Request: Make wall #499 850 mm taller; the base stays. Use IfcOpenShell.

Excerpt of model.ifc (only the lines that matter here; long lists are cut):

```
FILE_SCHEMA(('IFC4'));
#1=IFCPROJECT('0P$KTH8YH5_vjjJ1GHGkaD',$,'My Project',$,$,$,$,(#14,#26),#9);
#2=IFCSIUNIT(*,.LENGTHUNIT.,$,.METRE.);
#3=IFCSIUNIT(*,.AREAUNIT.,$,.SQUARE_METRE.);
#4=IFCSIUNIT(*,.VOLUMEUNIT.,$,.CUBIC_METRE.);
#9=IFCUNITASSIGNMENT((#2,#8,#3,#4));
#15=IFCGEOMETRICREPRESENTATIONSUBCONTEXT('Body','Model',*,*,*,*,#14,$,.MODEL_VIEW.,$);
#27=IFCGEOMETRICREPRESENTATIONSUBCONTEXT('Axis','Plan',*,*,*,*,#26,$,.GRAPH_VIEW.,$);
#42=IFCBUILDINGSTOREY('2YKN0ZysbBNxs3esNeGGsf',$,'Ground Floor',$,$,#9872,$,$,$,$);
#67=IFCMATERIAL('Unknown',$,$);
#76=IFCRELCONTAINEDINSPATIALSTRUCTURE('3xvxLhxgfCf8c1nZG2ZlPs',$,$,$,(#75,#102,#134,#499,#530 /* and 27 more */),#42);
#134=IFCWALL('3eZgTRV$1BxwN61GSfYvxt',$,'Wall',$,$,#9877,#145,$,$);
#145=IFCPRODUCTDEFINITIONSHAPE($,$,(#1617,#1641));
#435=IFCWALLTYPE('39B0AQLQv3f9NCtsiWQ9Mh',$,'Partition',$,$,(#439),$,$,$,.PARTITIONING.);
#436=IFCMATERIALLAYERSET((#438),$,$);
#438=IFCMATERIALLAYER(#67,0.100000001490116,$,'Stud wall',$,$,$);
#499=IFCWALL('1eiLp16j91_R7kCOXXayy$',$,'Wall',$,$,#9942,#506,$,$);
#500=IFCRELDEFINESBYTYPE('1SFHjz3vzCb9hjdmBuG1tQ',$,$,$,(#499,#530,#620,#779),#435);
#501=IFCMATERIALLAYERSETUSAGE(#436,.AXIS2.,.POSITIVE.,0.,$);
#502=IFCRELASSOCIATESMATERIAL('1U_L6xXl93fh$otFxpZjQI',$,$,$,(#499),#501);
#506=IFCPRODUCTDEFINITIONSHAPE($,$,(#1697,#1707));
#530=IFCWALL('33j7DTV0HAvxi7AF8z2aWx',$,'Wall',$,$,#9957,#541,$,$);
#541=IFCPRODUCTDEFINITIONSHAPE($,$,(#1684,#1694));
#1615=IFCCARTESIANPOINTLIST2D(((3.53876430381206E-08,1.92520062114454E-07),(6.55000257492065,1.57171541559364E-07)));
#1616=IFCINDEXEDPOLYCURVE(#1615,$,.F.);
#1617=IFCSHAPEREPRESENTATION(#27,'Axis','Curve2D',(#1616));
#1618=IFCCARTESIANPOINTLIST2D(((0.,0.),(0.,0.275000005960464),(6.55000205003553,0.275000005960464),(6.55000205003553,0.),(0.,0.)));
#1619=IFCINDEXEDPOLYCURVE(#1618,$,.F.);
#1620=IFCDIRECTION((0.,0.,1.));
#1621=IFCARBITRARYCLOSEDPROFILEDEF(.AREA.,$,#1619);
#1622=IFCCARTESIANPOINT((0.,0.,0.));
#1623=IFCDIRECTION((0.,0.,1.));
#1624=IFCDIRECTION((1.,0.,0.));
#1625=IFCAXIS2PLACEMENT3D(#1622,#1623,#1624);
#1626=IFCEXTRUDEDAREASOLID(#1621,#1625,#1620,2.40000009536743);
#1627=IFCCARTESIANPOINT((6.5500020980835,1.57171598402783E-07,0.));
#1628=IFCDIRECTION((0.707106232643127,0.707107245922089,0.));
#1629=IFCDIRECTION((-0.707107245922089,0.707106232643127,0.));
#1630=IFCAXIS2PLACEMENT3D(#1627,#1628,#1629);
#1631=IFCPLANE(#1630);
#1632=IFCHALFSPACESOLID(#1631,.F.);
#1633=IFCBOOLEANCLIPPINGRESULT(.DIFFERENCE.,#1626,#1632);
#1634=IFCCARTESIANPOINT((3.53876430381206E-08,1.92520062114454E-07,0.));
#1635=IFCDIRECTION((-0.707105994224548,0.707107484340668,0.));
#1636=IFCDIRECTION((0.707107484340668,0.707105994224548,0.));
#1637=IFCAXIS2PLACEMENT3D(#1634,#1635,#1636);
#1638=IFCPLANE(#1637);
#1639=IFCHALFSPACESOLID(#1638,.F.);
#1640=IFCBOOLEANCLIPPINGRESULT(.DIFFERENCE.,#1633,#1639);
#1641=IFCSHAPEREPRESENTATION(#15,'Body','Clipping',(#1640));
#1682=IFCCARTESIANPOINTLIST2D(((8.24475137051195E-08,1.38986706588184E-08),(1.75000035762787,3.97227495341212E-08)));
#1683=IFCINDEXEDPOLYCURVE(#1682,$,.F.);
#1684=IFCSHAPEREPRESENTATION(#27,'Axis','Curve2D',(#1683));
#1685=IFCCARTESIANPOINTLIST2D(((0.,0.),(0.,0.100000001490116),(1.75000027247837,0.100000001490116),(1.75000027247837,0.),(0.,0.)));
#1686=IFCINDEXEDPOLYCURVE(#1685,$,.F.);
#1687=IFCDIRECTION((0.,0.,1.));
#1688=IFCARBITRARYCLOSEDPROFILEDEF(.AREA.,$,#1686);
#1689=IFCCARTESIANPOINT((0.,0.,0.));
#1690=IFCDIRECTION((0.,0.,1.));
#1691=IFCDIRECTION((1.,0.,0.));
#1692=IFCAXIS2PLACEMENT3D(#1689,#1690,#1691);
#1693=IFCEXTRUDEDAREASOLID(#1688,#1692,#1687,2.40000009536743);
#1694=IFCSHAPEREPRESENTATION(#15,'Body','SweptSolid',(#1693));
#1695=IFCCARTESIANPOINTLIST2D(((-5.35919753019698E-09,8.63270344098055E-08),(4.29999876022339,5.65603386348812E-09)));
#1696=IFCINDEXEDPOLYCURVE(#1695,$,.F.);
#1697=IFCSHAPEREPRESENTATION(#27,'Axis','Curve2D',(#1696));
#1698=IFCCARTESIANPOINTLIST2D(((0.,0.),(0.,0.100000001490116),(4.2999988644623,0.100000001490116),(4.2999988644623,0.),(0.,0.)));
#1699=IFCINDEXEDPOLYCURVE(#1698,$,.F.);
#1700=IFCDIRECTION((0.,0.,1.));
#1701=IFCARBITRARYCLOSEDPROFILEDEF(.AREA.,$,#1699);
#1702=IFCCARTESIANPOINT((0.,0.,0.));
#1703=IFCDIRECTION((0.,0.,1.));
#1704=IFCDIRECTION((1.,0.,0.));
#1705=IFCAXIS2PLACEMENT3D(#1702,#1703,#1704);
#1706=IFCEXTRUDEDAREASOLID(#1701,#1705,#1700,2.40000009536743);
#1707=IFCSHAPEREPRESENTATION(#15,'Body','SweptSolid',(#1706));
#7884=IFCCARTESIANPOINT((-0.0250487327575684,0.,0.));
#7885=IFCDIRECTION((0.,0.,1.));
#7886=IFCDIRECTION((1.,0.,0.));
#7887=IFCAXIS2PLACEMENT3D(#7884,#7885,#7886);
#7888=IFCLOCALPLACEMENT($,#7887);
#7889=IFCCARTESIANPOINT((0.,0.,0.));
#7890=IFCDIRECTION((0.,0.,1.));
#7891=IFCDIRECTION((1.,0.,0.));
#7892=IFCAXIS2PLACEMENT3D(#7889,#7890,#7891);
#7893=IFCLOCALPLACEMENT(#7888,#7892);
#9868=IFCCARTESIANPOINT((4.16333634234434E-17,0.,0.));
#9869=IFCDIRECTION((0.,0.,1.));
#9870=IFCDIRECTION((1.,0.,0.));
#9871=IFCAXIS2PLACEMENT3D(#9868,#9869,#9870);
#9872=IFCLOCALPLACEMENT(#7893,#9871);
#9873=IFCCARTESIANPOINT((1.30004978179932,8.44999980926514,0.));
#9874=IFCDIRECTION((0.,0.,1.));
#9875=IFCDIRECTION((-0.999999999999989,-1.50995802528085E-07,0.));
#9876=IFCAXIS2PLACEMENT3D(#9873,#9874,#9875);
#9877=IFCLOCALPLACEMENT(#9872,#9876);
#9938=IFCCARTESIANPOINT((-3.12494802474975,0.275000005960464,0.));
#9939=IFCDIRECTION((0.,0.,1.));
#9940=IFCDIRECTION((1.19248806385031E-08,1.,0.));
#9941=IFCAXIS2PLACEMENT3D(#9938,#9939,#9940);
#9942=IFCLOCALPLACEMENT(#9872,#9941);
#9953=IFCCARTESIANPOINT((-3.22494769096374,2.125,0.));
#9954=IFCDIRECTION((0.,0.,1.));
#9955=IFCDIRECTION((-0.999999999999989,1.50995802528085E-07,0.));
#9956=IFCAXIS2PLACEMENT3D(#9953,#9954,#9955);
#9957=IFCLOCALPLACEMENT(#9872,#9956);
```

```python
import ifcopenshell
import ifcopenshell.geom
import ifcopenshell.util.representation
import ifcopenshell.util.shape

model = ifcopenshell.open("model.ifc")
settings = ifcopenshell.geom.settings()


def volume(element):
    """Net volume in cubic metres, openings subtracted."""
    shape = ifcopenshell.geom.create_shape(settings, element)
    return ifcopenshell.util.shape.get_volume(shape.geometry)


wall = model.by_guid("1eiLp16j91_R7kCOXXayy$")
before = volume(wall)

body = ifcopenshell.util.representation.get_representation(wall, "Model", "Body")
solid = body.Items[0]
old_height = solid.Depth
solid.Depth += 0.85
after = volume(wall)

print(f"height {old_height:g} -> {solid.Depth:g}, volume {before:.3f} -> {after:.3f} m3")

model.write("model_updated.ifc")
```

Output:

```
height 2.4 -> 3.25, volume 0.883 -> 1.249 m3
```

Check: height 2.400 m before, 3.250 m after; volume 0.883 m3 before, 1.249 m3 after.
